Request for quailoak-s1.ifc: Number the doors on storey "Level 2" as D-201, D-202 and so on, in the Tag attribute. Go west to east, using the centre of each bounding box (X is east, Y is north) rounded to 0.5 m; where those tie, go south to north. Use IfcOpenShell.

First a look at what the model holds.

```python
import ifcopenshell
import ifcopenshell.util.element
import ifcopenshell.util.placement

model = ifcopenshell.open("quailoak-s1.ifc")
print(model.schema)
storey = next(s for s in model.by_type("IfcBuildingStorey") if s.Name == "Level 2")
doors = [e for e in ifcopenshell.util.element.get_decomposition(storey) if e.is_a("IfcDoor")]
for e in sorted(doors, key=lambda e: e.id()):
    origin = ifcopenshell.util.placement.get_local_placement(e.ObjectPlacement)[:3, 3]
    print(e.id(), e.Tag, e.Name, origin.round(2) + 0.0, sep=" | ")
```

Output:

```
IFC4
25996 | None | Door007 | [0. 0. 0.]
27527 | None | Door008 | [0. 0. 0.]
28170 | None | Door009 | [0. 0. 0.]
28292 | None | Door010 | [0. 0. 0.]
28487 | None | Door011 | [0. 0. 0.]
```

```python
import ifcopenshell
import ifcopenshell.geom
import ifcopenshell.util.element
import ifcopenshell.util.shape

model = ifcopenshell.open("quailoak-s1.ifc")
settings = ifcopenshell.geom.settings()
settings.set("use-world-coords", True)


def centre(element):
    shape = ifcopenshell.geom.create_shape(settings, element)
    return ifcopenshell.util.shape.get_bbox_centroid(shape.geometry)


storey = next(s for s in model.by_type("IfcBuildingStorey") if s.Name == "Level 2")
doors = [e for e in ifcopenshell.util.element.get_decomposition(storey) if e.is_a("IfcDoor")]

# Insertion points can sit at a corner or the storey origin, so sort by the geometry (in metres).
centres = {e: centre(e) for e in doors}
doors.sort(key=lambda e: (round(centres[e][0] / 0.5), centres[e][1]))

for i, e in enumerate(doors, start=1):
    number = f"D-2{i:02d}"
    e.Tag = number
    print(e.id(), number)

model.write("quailoak-s1_rev.ifc")
```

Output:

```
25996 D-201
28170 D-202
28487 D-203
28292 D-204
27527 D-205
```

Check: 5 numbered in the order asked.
